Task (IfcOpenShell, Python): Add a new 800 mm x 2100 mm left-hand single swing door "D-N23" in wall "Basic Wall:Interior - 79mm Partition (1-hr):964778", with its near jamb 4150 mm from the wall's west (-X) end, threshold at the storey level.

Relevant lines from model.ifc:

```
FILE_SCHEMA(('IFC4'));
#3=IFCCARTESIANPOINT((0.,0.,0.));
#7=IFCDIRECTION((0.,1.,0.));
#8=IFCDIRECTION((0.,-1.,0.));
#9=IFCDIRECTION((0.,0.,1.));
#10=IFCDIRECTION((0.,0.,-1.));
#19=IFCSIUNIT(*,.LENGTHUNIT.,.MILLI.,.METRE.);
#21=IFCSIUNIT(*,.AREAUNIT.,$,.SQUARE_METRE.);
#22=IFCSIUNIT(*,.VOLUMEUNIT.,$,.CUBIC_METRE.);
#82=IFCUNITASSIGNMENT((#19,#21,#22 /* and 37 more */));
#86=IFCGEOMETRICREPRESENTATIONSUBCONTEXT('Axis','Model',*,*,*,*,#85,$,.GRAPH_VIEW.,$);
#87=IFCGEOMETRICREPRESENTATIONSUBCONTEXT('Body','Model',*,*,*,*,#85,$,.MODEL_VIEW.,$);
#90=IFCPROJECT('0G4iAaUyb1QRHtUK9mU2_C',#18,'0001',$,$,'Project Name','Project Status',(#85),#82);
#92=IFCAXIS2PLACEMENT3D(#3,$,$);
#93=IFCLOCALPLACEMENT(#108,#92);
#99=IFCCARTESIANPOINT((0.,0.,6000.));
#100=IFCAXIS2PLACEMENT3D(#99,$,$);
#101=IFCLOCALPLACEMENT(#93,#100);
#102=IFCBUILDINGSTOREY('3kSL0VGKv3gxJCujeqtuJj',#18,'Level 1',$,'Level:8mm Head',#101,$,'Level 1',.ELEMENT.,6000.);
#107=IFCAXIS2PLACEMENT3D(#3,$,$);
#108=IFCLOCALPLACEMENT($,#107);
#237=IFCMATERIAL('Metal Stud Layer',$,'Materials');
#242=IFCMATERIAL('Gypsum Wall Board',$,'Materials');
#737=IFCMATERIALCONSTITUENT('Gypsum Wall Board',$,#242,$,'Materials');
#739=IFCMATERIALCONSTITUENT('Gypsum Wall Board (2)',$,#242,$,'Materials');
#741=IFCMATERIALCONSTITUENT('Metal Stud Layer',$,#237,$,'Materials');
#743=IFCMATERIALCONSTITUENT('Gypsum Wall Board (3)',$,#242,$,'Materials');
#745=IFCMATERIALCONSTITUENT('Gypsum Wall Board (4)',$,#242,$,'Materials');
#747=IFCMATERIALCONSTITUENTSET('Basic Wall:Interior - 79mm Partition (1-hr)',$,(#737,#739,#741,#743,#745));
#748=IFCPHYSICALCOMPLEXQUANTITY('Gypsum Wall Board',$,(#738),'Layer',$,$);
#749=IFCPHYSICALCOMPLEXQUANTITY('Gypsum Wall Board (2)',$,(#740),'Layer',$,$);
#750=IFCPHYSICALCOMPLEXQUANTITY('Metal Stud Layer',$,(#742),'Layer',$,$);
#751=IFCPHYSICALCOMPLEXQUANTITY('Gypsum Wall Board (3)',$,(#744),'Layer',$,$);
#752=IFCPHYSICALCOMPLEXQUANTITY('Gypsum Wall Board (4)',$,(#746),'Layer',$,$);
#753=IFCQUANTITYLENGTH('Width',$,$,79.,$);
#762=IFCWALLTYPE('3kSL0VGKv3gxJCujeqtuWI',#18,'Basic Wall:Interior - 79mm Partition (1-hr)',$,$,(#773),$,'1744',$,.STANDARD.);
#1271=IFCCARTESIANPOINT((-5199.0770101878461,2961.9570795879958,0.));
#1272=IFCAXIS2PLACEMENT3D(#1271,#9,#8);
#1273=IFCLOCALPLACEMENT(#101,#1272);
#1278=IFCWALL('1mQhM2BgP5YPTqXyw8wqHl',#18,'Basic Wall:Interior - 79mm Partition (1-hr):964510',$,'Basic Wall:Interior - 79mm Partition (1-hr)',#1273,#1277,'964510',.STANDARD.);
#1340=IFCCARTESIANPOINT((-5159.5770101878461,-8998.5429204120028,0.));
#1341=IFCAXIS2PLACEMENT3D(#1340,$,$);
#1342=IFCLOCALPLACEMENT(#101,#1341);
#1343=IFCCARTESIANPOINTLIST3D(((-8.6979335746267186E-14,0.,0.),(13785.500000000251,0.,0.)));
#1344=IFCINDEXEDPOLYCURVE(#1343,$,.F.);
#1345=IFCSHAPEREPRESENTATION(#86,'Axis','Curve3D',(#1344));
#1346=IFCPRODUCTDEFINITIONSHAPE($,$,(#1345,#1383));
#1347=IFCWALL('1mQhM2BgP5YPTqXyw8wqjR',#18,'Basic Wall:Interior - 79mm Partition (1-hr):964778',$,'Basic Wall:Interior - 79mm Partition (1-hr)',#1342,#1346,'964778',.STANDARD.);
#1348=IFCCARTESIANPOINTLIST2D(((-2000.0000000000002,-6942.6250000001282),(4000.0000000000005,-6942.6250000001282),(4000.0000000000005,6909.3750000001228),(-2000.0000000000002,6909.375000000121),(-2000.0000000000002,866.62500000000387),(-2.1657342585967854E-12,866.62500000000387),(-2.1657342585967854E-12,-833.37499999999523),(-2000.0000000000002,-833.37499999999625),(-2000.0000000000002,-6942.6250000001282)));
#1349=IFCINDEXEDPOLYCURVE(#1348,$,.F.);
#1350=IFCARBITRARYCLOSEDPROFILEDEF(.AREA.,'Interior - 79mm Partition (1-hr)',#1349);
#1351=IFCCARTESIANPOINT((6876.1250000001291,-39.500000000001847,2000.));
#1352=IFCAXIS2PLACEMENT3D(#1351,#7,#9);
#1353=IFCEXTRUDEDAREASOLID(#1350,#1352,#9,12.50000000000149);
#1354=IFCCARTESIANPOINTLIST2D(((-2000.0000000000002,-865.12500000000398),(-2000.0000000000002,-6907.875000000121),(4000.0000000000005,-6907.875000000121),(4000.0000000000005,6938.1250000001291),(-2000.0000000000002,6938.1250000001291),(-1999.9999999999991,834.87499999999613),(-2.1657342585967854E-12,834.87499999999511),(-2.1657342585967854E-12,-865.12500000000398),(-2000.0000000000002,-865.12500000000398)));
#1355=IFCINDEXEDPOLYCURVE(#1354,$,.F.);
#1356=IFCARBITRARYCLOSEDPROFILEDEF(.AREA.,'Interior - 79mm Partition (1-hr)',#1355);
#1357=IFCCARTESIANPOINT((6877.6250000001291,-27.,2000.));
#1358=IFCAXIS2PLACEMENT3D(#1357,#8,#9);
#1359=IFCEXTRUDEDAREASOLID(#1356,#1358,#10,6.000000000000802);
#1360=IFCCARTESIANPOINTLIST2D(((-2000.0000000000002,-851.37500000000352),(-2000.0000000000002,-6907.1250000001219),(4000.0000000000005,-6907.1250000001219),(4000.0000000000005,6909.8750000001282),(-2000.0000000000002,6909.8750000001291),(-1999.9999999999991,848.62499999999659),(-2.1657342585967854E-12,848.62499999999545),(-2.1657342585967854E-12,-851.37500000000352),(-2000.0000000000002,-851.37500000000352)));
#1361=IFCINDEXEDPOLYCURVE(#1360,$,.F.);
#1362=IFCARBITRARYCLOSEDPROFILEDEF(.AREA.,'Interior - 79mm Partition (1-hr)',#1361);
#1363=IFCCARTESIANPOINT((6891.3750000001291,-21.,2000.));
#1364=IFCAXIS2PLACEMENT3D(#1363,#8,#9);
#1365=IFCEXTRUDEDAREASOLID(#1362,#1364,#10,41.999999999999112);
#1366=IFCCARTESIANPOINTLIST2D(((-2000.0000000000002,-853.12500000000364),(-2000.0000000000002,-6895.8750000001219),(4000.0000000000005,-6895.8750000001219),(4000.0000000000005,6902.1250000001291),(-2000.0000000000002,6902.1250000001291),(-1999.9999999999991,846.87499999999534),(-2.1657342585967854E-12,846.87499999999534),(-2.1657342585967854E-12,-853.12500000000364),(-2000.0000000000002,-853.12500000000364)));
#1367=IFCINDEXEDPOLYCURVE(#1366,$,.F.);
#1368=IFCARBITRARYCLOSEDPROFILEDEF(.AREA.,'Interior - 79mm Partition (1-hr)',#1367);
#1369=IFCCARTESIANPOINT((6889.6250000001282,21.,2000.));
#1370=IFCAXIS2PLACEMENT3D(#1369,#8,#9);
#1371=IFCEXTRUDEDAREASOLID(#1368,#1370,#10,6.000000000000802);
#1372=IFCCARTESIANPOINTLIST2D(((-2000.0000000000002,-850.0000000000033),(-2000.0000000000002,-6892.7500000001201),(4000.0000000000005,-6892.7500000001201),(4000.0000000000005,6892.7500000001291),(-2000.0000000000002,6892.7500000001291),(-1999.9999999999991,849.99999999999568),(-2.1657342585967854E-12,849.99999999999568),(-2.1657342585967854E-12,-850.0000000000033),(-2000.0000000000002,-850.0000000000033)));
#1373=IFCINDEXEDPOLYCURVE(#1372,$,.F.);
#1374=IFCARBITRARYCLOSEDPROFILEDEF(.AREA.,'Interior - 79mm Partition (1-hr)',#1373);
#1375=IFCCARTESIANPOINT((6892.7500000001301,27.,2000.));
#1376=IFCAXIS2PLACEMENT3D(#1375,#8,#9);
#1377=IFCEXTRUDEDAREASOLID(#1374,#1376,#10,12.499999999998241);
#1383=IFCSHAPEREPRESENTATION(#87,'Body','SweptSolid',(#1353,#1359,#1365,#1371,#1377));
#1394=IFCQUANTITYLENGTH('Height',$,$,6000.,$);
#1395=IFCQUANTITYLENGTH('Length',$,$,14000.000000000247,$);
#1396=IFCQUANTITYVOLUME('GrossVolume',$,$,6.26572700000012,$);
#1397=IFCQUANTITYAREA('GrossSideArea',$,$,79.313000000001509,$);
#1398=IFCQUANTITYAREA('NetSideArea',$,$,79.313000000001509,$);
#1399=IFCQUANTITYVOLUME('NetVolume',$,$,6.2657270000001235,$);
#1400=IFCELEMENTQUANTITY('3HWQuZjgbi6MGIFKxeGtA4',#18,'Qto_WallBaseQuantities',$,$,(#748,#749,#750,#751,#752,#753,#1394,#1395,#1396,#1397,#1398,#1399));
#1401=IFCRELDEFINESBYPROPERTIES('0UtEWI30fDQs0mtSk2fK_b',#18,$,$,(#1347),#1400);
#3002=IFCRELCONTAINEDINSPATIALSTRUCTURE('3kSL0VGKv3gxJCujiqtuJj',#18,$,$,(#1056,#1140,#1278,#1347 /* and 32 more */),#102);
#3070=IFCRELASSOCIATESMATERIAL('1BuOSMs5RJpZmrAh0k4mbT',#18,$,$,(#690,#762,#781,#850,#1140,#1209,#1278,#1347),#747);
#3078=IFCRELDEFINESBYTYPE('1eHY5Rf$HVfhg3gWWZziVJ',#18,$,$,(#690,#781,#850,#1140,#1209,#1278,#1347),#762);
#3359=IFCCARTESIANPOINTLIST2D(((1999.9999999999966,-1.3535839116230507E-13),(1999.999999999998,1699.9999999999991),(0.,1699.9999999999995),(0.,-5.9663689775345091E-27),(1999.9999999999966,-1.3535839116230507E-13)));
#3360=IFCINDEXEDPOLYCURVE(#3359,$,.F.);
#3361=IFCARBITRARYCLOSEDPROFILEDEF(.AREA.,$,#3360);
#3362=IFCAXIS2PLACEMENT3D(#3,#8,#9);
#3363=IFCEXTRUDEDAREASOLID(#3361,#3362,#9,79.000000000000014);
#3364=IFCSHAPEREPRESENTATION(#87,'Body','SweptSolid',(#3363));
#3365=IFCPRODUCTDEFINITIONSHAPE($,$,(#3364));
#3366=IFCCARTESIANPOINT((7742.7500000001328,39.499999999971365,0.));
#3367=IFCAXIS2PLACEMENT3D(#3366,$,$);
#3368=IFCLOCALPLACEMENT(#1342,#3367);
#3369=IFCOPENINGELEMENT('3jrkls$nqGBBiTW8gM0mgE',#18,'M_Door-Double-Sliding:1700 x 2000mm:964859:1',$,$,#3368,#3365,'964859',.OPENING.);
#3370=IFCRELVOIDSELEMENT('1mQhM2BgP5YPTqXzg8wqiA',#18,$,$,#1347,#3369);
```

```python
import numpy as np
import ifcopenshell
import ifcopenshell.api.feature
import ifcopenshell.api.geometry
import ifcopenshell.api.pset
import ifcopenshell.api.root
import ifcopenshell.api.spatial
import ifcopenshell.geom
import ifcopenshell.util.element
import ifcopenshell.util.placement
import ifcopenshell.util.representation
import ifcopenshell.util.shape
import ifcopenshell.util.unit

model = ifcopenshell.open("model.ifc")
unit_scale = ifcopenshell.util.unit.calculate_unit_scale(model)
area_scale = ifcopenshell.util.unit.calculate_unit_scale(model, "AREAUNIT")
volume_scale = ifcopenshell.util.unit.calculate_unit_scale(model, "VOLUMEUNIT")
settings = ifcopenshell.geom.settings()


def volume(element):
    """Net volume in cubic metres, openings subtracted."""
    shape = ifcopenshell.geom.create_shape(settings, element)
    return ifcopenshell.util.shape.get_volume(shape.geometry)


wall = model.by_guid("1mQhM2BgP5YPTqXyw8wqjR")
storey = ifcopenshell.util.element.get_container(wall, ifc_class="IfcBuildingStorey")
context = ifcopenshell.util.representation.get_context(model, "Model", "Body", "MODEL_VIEW")
before = volume(wall)

width, height, from_end, sill = 0.8, 2.1, 4.15, 0.0  # metres

# The wall runs along its own X axis, and the end named is its -X end.
wall_shape = ifcopenshell.geom.create_shape(settings, wall)
x, y, z = ifcopenshell.util.shape.get_vertices(wall_shape.geometry).T
start = x.min() + from_end
face, thickness = float(y.min()), float(y.max() - y.min())
wall_matrix = ifcopenshell.util.placement.get_local_placement(wall.ObjectPlacement)
level = ifcopenshell.util.placement.get_local_placement(storey.ObjectPlacement)[2, 3]


def in_wall(x, y):
    """Placement at x, y metres in the wall's axes, at sill height."""
    matrix = wall_matrix.copy()
    matrix[:, 3] = wall_matrix @ np.array([x / unit_scale, y / unit_scale, 0.0, 1.0])
    matrix[2, 3] = level + sill / unit_scale
    return matrix


# Opening: a box that overshoots both wall faces by 50 mm.
opening = ifcopenshell.api.root.create_entity(model, ifc_class="IfcOpeningElement", predefined_type="OPENING")
box = ifcopenshell.api.geometry.add_wall_representation(
    model, context=context, length=width, height=height, thickness=thickness + 0.1
)
ifcopenshell.api.geometry.assign_representation(model, product=opening, representation=box)
ifcopenshell.api.geometry.edit_object_placement(model, product=opening, matrix=in_wall(start, face - 0.05), is_si=False)
ifcopenshell.api.feature.add_feature(model, feature=opening, element=wall)

door = ifcopenshell.api.root.create_entity(model, ifc_class="IfcDoor", name="D-N23", predefined_type="DOOR")
door.OverallWidth, door.OverallHeight = width / unit_scale, height / unit_scale
door.OperationType = "SINGLE_SWING_LEFT"
body = ifcopenshell.api.geometry.add_door_representation(
    model,
    context=context,
    overall_width=door.OverallWidth,
    overall_height=door.OverallHeight,
    operation_type="SINGLE_SWING_LEFT",
    lining_properties={"LiningDepth": thickness / unit_scale, "ThresholdDepth": thickness / unit_scale},
)
ifcopenshell.api.geometry.assign_representation(model, product=door, representation=body)
ifcopenshell.api.spatial.assign_container(model, products=[door], relating_structure=storey)
ifcopenshell.api.feature.add_filling(model, opening=opening, element=door)

# The lining spans the wall, so the door starts at the wall face.
ifcopenshell.api.geometry.edit_object_placement(model, product=door, matrix=in_wall(start, face), is_si=False)

after = volume(wall)

# Update the wall's stored quantities.
qto = model.by_id(ifcopenshell.util.element.get_pset(wall, "Qto_WallBaseQuantities", should_inherit=False)["id"])
ifcopenshell.api.pset.edit_qto(model, qto=qto, properties={
    "NetSideArea": after / thickness / area_scale,
    "NetVolume": after / volume_scale,
})

print(f"wall volume {before:.3f} -> {after:.3f} m3")

model.write("model_edited.ifc")
```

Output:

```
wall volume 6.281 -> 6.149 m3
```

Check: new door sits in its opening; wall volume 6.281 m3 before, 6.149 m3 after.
